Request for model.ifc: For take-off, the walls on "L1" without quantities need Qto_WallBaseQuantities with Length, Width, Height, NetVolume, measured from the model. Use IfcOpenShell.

First a look at what the model holds.

```python
import ifcopenshell
import ifcopenshell.util.element
import ifcopenshell.util.unit

model = ifcopenshell.open("model.ifc")
print(model.schema)
for unit_type in ("LENGTHUNIT", "AREAUNIT", "VOLUMEUNIT"):
    print(unit_type, ifcopenshell.util.unit.calculate_unit_scale(model, unit_type))
storey = next(s for s in model.by_type("IfcBuildingStorey") if s.Name == "L1")
walls = [e for e in ifcopenshell.util.element.get_decomposition(storey) if e.is_a("IfcWall")]
for e in sorted(walls, key=lambda e: e.id()):
    print(e.id(), e.is_a(), e.Name, list(ifcopenshell.util.element.get_psets(e, qtos_only=True)), sep=" | ")
```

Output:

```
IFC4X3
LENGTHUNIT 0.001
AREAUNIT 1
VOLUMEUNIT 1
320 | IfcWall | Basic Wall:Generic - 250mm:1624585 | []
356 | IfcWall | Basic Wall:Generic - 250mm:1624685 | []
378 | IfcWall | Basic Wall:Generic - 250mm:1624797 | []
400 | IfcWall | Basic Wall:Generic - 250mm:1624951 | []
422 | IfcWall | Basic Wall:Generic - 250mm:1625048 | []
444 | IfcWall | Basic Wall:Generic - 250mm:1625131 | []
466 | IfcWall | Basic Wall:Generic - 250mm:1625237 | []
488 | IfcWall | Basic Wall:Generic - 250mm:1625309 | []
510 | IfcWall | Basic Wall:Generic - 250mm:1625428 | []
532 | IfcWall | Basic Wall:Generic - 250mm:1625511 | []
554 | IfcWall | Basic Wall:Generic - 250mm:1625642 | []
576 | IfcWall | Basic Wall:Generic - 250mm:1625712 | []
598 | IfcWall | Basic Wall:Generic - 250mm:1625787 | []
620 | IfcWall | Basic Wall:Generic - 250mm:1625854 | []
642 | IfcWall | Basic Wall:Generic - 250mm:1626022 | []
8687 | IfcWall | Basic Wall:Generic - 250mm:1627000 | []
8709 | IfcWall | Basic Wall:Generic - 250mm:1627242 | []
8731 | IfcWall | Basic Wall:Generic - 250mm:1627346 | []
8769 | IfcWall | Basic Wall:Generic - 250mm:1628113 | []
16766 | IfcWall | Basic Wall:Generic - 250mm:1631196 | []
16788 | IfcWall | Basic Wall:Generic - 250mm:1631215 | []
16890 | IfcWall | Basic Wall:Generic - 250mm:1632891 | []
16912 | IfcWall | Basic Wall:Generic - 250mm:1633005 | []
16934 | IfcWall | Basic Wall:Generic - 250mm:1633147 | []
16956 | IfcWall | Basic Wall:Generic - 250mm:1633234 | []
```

```python
import ifcopenshell
import ifcopenshell.api.pset
import ifcopenshell.geom
import ifcopenshell.util.element
import ifcopenshell.util.shape
import ifcopenshell.util.unit

model = ifcopenshell.open("model.ifc")
unit_scale = ifcopenshell.util.unit.calculate_unit_scale(model)
volume_scale = ifcopenshell.util.unit.calculate_unit_scale(model, "VOLUMEUNIT")
settings = ifcopenshell.geom.settings()

storey = next(s for s in model.by_type("IfcBuildingStorey") if s.Name == "L1")
walls = [e for e in ifcopenshell.util.element.get_decomposition(storey) if e.is_a("IfcWall")]

for e in sorted(walls, key=lambda e: e.id()):
    if ifcopenshell.util.element.get_psets(e, qtos_only=True, should_inherit=False):
        continue
    # Geometry comes back in metres, in the element's own axes.
    shape = ifcopenshell.geom.create_shape(settings, e)
    values = {
        "Length": ifcopenshell.util.shape.get_x(shape.geometry) / unit_scale,
        "Width": ifcopenshell.util.shape.get_y(shape.geometry) / unit_scale,
        "Height": ifcopenshell.util.shape.get_z(shape.geometry) / unit_scale,
        "NetVolume": ifcopenshell.util.shape.get_volume(shape.geometry) / volume_scale,
    }
    qto = ifcopenshell.api.pset.add_qto(model, product=e, name="Qto_WallBaseQuantities")
    ifcopenshell.api.pset.edit_qto(model, qto=qto, properties=values)
    print(e.id(), {k: round(v, 3) for k, v in values.items()})

model.write("model-out.ifc")
```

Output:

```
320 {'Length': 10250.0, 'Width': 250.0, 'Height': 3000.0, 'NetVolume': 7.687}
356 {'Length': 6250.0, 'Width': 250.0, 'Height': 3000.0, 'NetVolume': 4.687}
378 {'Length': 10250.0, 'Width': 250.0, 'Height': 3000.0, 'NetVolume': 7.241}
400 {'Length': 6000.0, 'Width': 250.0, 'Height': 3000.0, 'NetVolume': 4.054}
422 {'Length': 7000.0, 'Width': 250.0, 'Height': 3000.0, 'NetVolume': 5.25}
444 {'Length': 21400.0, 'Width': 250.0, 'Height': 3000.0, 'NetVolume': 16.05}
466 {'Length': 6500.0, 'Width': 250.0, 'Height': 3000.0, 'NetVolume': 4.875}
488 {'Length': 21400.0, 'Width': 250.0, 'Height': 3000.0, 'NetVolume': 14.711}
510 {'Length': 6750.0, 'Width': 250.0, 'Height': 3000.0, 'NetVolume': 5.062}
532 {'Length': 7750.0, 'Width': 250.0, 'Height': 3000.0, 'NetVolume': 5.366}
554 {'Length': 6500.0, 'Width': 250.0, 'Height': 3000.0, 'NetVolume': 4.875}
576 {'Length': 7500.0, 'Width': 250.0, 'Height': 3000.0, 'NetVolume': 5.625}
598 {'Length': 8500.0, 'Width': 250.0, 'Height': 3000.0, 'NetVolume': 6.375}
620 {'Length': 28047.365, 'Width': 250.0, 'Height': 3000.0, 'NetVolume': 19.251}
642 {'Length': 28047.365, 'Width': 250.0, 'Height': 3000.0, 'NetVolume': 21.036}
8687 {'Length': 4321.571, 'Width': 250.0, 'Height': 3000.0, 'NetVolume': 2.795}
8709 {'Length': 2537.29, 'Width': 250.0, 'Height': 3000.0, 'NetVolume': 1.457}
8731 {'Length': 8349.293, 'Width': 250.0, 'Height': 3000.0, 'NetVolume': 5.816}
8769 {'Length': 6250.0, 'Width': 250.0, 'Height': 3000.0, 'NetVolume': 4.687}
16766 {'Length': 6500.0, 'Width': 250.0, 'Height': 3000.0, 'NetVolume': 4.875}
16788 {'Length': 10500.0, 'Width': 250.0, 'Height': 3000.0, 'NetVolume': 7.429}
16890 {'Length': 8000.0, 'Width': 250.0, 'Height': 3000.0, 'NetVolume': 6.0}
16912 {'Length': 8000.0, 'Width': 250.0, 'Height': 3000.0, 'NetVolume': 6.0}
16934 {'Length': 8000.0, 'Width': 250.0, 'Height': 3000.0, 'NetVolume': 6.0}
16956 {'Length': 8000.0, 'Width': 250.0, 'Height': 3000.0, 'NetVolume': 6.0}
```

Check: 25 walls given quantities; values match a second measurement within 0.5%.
